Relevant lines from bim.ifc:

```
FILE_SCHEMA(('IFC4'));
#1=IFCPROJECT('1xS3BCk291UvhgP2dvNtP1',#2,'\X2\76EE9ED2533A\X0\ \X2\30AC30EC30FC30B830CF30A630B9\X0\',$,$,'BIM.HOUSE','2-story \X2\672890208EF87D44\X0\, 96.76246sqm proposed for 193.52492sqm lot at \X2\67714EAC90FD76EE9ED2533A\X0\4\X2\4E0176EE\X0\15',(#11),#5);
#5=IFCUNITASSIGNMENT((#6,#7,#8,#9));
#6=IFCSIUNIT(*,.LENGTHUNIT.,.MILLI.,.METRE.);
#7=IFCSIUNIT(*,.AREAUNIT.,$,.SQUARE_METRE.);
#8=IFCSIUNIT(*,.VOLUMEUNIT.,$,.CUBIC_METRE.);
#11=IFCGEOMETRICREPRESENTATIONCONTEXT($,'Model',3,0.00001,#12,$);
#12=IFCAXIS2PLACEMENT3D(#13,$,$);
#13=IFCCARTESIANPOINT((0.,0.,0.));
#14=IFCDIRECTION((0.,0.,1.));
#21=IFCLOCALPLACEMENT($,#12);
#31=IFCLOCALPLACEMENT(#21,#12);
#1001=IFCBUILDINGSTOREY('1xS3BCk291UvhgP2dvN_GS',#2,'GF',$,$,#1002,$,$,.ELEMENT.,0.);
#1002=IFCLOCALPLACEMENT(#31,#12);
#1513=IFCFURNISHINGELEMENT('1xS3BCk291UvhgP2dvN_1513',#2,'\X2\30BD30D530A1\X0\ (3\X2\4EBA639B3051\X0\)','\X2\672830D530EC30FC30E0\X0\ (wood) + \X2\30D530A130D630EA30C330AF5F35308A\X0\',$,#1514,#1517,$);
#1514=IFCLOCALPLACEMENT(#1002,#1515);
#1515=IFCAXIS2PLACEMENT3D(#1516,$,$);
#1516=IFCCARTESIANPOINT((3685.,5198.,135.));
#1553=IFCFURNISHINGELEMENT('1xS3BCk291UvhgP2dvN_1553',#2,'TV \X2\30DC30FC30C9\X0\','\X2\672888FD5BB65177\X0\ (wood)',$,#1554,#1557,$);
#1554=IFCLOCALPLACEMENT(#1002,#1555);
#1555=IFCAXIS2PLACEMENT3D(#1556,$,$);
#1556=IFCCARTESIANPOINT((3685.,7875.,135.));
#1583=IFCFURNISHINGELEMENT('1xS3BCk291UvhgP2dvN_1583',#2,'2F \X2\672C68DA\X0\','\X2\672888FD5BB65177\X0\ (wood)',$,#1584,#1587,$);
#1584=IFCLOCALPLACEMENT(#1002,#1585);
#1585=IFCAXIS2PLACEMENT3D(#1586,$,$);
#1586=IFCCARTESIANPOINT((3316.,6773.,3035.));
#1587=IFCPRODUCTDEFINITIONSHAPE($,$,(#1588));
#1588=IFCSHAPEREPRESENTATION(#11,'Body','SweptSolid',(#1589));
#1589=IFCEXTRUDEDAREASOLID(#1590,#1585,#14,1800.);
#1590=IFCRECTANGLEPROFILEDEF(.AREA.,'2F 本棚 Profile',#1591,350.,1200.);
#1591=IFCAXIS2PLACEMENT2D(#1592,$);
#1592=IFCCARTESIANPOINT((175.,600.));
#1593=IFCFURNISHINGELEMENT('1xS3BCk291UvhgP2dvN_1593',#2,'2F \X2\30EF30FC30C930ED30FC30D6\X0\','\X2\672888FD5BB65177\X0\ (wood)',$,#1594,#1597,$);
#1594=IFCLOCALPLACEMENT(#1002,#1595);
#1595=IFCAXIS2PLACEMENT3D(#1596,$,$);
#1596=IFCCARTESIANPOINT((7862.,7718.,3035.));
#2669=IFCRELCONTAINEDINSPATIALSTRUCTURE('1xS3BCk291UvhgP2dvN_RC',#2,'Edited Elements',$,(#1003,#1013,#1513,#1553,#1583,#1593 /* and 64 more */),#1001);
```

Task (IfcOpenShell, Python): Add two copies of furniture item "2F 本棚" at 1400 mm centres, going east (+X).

```python
import numpy as np
import ifcopenshell
import ifcopenshell.api.geometry
import ifcopenshell.api.root
import ifcopenshell.util.element
import ifcopenshell.util.placement
import ifcopenshell.util.unit

model = ifcopenshell.open("bim.ifc")
unit_scale = ifcopenshell.util.unit.calculate_unit_scale(model)


def reuse_history(source, copy):
    """copy_class also copies each property set's owner history, people and application; keep the originals."""
    for rel in copy.IsDefinedBy:
        if rel.is_a("IfcRelDefinesByProperties") and (history := rel.RelatingPropertyDefinition.OwnerHistory):
            rel.RelatingPropertyDefinition.OwnerHistory = source.OwnerHistory
            ifcopenshell.util.element.remove_deep2(model, history)


source = model.by_id(1583)
base = ifcopenshell.util.placement.get_local_placement(source.ObjectPlacement)
step = np.array([1.0, 0.0, 0.0]) * 1.4 / unit_scale

for i in range(1, 3):
    copy = ifcopenshell.api.root.copy_class(model, product=source)
    copy.Representation = ifcopenshell.util.element.copy_deep(
        model, source.Representation, exclude=["IfcGeometricRepresentationContext", "IfcRepresentationMap"]
    )
    reuse_history(source, copy)
    matrix = base.copy()
    matrix[:3, 3] += i * step
    print("added at", matrix[:3, 3].round(3) + 0.0)
    ifcopenshell.api.geometry.edit_object_placement(model, product=copy, matrix=matrix, is_si=False)

model.write("bim_updated.ifc")
```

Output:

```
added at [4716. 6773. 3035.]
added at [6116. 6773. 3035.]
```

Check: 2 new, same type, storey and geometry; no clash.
